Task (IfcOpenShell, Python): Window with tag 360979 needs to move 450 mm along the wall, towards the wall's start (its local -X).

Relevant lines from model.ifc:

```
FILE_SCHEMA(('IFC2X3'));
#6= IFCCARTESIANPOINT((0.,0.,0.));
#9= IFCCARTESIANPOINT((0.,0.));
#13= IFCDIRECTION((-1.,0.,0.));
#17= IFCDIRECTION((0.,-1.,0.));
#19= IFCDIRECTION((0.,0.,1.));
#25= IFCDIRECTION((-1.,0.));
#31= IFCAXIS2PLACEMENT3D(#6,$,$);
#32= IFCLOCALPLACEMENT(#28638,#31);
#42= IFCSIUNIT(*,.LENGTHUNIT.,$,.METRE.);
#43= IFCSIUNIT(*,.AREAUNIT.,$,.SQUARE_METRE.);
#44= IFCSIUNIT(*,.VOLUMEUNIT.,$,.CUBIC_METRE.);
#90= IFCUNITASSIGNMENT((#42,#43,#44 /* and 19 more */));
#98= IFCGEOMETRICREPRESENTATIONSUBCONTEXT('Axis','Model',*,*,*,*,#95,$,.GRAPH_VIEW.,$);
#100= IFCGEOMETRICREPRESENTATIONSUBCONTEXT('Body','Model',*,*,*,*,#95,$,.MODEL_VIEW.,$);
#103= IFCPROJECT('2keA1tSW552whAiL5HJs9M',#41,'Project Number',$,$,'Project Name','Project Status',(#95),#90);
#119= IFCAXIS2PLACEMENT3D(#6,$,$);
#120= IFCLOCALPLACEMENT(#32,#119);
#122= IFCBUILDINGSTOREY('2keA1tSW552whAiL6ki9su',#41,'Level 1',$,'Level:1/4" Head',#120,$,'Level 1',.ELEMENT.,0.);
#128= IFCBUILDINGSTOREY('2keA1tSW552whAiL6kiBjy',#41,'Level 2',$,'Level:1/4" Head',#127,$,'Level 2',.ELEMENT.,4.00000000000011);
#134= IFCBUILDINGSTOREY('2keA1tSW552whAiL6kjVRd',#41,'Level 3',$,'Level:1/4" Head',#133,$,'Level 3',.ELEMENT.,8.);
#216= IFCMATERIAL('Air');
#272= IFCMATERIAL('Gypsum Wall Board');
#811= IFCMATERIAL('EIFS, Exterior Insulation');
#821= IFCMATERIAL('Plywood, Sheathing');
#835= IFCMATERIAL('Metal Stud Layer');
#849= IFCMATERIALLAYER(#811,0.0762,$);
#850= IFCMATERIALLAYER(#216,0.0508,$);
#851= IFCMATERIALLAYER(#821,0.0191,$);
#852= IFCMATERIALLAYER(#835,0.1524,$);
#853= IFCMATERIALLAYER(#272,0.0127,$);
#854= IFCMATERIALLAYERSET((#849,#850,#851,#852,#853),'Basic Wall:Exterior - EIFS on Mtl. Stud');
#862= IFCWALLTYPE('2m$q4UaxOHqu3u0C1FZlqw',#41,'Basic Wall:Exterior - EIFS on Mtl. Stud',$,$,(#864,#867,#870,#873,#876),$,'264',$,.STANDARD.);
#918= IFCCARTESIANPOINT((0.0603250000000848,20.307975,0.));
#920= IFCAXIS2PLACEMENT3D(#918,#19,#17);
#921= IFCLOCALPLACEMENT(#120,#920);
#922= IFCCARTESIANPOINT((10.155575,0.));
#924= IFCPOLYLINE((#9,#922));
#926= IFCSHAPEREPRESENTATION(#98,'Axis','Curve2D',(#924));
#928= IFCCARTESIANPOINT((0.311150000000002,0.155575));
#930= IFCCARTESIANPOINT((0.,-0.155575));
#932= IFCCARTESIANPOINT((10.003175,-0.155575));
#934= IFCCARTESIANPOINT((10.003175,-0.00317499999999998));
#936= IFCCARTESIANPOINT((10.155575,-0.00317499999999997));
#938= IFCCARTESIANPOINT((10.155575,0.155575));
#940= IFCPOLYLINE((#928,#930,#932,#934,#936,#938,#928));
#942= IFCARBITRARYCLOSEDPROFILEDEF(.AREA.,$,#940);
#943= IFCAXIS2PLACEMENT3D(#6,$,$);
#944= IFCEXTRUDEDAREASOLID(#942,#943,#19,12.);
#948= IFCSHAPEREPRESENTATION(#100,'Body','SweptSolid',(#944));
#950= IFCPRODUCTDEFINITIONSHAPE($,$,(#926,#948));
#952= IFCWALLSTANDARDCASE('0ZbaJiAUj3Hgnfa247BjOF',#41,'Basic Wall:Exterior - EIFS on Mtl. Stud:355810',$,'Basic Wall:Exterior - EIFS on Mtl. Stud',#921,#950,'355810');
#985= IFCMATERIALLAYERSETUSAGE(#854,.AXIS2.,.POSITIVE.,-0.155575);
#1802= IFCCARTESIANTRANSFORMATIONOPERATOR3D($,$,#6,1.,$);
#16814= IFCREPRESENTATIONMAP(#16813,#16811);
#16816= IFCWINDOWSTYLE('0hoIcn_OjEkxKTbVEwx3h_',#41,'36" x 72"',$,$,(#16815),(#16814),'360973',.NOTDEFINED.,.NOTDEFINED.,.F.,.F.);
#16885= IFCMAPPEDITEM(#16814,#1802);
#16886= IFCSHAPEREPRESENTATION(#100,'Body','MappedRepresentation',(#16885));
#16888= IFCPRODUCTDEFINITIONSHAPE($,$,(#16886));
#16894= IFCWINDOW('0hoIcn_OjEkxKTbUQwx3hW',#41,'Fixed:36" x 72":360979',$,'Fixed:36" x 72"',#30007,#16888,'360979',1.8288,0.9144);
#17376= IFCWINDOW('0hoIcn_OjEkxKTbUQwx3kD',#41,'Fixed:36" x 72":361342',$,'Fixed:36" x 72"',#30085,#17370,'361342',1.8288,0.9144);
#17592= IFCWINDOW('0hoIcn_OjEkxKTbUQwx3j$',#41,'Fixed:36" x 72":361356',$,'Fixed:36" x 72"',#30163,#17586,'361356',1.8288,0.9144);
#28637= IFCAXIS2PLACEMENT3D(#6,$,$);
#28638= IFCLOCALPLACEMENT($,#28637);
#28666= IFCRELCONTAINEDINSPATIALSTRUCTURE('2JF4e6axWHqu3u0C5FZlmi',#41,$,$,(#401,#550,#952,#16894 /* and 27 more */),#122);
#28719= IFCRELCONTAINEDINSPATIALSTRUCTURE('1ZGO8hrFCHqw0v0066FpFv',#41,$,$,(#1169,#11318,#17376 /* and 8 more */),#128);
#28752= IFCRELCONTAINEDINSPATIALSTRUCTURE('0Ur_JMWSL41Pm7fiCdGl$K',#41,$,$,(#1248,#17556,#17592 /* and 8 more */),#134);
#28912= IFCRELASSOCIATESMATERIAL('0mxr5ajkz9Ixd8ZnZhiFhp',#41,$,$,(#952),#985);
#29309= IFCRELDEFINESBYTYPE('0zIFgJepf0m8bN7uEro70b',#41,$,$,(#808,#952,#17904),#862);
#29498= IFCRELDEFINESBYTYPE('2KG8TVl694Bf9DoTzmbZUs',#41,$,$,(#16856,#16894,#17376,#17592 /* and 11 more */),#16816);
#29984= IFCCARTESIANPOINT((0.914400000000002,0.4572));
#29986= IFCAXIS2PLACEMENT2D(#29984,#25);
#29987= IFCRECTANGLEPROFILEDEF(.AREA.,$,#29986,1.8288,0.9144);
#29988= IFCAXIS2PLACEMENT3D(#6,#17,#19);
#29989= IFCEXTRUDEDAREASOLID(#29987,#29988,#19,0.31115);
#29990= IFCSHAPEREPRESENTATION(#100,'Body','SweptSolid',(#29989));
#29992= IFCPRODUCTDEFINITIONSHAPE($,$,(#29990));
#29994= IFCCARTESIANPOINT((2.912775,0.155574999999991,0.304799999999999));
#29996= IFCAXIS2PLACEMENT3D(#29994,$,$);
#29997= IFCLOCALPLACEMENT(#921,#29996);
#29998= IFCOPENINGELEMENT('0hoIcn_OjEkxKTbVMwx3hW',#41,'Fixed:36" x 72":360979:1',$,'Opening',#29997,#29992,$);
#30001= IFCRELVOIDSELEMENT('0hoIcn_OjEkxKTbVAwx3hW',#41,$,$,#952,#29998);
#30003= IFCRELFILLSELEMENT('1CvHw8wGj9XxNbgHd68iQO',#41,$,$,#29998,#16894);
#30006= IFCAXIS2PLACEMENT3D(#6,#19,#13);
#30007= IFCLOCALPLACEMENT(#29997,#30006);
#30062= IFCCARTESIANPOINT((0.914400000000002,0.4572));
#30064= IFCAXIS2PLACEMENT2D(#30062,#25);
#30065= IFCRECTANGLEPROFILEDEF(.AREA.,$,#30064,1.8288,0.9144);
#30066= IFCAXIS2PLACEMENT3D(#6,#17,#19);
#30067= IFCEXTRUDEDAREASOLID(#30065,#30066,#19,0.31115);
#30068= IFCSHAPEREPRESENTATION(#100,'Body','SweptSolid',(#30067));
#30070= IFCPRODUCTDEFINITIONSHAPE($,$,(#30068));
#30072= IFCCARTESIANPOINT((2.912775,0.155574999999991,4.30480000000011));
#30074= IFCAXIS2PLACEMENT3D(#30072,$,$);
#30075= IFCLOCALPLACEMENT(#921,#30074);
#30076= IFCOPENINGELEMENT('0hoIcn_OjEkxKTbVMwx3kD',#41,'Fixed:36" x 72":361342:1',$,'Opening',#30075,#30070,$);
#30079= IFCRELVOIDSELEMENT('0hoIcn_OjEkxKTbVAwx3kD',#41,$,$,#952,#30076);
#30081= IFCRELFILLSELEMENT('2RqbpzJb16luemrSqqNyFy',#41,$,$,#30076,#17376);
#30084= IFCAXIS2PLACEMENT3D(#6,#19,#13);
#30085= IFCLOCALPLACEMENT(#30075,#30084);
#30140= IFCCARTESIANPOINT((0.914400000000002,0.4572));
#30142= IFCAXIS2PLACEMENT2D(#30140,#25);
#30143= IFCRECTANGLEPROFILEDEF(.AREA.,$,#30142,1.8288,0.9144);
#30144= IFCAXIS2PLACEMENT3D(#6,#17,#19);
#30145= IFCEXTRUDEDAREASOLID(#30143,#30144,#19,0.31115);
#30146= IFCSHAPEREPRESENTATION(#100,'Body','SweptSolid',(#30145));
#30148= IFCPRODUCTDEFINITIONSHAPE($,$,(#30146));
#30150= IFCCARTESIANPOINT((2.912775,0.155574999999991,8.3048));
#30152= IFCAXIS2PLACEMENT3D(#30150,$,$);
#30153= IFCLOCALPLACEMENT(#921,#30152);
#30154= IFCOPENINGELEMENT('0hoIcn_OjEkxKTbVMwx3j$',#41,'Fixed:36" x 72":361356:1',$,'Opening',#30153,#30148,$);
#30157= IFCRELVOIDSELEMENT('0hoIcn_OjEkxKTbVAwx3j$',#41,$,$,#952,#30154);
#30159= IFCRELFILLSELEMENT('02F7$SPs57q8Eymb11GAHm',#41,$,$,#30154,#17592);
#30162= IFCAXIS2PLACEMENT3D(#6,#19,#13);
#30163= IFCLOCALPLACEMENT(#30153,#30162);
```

```python
import ifcopenshell
import ifcopenshell.api.geometry
import ifcopenshell.util.placement
import ifcopenshell.util.unit

model = ifcopenshell.open("model.ifc")
unit_scale = ifcopenshell.util.unit.calculate_unit_scale(model)

window = model.by_guid("0hoIcn_OjEkxKTbUQwx3hW")
opening = window.FillsVoids[0].RelatingOpeningElement
wall = opening.VoidsElements[0].RelatingBuildingElement

wall_matrix = ifcopenshell.util.placement.get_local_placement(wall.ObjectPlacement)
shift = wall_matrix[:3, 0] * -0.45 / unit_scale
before = ifcopenshell.util.placement.get_local_placement(window.ObjectPlacement)[:3, 3].copy()

# The window is placed relative to its opening, so it follows when the opening moves.
matrix = ifcopenshell.util.placement.get_local_placement(opening.ObjectPlacement)
matrix[:3, 3] += shift
ifcopenshell.api.geometry.edit_object_placement(
    model, product=opening, matrix=matrix, is_si=False, should_transform_children=True
)

after = ifcopenshell.util.placement.get_local_placement(window.ObjectPlacement)[:3, 3]
print("window moved by", (after - before).round(3) + 0.0)

model.write("model_edited.ifc")
```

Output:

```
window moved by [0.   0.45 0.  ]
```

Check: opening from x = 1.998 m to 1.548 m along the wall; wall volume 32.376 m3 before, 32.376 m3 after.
